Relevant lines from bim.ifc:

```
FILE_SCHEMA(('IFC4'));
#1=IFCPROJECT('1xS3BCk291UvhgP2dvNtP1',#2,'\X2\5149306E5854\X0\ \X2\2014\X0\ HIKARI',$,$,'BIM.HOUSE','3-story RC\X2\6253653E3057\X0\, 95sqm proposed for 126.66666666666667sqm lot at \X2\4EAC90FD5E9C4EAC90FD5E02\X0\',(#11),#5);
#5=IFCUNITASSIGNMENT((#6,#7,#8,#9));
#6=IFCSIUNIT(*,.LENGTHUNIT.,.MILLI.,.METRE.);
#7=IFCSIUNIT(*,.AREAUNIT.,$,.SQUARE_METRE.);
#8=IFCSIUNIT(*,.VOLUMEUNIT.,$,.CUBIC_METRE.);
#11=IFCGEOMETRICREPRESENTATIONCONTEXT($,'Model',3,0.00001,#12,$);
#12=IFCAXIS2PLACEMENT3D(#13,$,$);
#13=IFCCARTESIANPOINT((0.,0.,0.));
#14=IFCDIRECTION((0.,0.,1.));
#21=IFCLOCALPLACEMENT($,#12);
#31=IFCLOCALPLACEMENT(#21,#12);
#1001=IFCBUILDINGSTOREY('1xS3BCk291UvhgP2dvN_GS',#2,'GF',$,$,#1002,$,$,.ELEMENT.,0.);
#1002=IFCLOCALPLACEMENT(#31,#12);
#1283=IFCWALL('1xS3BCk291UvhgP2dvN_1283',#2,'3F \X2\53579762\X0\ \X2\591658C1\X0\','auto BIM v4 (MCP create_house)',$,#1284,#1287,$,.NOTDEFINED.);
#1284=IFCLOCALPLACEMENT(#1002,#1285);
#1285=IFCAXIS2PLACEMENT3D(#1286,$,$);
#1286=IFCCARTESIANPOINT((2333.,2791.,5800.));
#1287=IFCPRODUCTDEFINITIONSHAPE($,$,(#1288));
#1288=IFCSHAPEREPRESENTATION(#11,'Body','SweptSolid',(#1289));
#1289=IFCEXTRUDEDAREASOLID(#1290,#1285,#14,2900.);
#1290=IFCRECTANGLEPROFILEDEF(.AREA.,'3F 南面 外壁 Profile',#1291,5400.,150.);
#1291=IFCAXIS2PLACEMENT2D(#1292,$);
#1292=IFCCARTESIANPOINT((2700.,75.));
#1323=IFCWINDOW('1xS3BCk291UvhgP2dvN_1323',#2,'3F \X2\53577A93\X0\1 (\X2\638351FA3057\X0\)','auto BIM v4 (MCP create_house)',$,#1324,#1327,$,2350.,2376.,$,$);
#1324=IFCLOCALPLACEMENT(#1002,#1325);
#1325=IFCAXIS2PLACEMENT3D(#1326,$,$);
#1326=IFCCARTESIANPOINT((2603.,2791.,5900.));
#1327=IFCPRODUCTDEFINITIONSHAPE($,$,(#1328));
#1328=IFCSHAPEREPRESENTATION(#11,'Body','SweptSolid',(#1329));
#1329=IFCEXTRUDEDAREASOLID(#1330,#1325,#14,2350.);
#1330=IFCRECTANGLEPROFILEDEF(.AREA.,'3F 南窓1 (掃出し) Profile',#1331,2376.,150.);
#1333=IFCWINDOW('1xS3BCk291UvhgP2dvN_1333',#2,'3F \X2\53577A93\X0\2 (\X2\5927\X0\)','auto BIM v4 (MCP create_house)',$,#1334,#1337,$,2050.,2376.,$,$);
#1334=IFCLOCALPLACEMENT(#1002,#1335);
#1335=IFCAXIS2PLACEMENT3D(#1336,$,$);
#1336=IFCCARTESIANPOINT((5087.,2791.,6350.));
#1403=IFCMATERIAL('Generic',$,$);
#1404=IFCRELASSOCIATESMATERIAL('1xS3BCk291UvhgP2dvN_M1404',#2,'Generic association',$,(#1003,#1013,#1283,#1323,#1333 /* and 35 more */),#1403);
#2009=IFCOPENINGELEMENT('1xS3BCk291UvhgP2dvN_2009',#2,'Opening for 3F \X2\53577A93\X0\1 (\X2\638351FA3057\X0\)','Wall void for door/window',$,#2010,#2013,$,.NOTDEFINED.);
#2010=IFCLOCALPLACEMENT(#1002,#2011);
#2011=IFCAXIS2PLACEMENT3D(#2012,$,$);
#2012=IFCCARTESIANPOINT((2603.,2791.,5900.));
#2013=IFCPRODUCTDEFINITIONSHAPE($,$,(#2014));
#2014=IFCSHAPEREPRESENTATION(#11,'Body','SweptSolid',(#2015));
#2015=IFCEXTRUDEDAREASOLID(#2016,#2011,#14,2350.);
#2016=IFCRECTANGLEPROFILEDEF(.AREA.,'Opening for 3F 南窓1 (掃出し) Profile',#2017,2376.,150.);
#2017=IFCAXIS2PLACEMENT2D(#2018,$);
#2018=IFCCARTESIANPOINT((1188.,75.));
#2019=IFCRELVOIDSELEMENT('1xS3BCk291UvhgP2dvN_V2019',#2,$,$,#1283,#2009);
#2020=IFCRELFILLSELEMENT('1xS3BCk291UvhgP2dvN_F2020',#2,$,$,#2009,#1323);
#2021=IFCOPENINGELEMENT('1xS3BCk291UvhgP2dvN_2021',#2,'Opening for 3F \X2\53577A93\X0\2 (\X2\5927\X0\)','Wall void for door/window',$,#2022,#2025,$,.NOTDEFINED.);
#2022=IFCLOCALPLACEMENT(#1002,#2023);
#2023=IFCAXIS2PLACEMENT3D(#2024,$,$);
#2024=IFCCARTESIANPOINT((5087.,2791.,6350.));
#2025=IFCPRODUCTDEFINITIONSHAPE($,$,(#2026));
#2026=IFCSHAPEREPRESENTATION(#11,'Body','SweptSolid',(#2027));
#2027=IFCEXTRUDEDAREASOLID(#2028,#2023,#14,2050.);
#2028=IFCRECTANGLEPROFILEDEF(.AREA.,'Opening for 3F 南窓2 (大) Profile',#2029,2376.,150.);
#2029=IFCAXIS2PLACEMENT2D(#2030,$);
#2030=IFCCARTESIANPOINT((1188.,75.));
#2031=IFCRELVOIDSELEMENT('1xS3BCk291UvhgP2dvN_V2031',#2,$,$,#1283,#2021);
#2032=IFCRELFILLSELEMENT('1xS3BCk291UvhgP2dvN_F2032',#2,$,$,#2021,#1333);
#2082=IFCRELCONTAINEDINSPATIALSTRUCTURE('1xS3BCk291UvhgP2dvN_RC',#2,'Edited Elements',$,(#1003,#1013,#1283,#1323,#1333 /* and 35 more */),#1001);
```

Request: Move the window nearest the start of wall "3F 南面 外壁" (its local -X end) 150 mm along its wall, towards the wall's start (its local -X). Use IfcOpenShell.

```python
import ifcopenshell
import ifcopenshell.api.geometry
import ifcopenshell.util.placement
import ifcopenshell.util.unit

model = ifcopenshell.open("bim.ifc")
unit_scale = ifcopenshell.util.unit.calculate_unit_scale(model)

window = model.by_id(1323)
opening = window.FillsVoids[0].RelatingOpeningElement
wall = opening.VoidsElements[0].RelatingBuildingElement

wall_matrix = ifcopenshell.util.placement.get_local_placement(wall.ObjectPlacement)
shift = wall_matrix[:3, 0] * -0.15 / unit_scale
before = ifcopenshell.util.placement.get_local_placement(window.ObjectPlacement)[:3, 3].copy()

# The window is not placed relative to its opening, so move both.
for product in (opening, window):
    matrix = ifcopenshell.util.placement.get_local_placement(product.ObjectPlacement)
    matrix[:3, 3] += shift
    ifcopenshell.api.geometry.edit_object_placement(model, product=product, matrix=matrix, is_si=False)

after = ifcopenshell.util.placement.get_local_placement(window.ObjectPlacement)[:3, 3]
print("window moved by", (after - before).round(3) + 0.0)

model.write("bim_rev.ifc")
```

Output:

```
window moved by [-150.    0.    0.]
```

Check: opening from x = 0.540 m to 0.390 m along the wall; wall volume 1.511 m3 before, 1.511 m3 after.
